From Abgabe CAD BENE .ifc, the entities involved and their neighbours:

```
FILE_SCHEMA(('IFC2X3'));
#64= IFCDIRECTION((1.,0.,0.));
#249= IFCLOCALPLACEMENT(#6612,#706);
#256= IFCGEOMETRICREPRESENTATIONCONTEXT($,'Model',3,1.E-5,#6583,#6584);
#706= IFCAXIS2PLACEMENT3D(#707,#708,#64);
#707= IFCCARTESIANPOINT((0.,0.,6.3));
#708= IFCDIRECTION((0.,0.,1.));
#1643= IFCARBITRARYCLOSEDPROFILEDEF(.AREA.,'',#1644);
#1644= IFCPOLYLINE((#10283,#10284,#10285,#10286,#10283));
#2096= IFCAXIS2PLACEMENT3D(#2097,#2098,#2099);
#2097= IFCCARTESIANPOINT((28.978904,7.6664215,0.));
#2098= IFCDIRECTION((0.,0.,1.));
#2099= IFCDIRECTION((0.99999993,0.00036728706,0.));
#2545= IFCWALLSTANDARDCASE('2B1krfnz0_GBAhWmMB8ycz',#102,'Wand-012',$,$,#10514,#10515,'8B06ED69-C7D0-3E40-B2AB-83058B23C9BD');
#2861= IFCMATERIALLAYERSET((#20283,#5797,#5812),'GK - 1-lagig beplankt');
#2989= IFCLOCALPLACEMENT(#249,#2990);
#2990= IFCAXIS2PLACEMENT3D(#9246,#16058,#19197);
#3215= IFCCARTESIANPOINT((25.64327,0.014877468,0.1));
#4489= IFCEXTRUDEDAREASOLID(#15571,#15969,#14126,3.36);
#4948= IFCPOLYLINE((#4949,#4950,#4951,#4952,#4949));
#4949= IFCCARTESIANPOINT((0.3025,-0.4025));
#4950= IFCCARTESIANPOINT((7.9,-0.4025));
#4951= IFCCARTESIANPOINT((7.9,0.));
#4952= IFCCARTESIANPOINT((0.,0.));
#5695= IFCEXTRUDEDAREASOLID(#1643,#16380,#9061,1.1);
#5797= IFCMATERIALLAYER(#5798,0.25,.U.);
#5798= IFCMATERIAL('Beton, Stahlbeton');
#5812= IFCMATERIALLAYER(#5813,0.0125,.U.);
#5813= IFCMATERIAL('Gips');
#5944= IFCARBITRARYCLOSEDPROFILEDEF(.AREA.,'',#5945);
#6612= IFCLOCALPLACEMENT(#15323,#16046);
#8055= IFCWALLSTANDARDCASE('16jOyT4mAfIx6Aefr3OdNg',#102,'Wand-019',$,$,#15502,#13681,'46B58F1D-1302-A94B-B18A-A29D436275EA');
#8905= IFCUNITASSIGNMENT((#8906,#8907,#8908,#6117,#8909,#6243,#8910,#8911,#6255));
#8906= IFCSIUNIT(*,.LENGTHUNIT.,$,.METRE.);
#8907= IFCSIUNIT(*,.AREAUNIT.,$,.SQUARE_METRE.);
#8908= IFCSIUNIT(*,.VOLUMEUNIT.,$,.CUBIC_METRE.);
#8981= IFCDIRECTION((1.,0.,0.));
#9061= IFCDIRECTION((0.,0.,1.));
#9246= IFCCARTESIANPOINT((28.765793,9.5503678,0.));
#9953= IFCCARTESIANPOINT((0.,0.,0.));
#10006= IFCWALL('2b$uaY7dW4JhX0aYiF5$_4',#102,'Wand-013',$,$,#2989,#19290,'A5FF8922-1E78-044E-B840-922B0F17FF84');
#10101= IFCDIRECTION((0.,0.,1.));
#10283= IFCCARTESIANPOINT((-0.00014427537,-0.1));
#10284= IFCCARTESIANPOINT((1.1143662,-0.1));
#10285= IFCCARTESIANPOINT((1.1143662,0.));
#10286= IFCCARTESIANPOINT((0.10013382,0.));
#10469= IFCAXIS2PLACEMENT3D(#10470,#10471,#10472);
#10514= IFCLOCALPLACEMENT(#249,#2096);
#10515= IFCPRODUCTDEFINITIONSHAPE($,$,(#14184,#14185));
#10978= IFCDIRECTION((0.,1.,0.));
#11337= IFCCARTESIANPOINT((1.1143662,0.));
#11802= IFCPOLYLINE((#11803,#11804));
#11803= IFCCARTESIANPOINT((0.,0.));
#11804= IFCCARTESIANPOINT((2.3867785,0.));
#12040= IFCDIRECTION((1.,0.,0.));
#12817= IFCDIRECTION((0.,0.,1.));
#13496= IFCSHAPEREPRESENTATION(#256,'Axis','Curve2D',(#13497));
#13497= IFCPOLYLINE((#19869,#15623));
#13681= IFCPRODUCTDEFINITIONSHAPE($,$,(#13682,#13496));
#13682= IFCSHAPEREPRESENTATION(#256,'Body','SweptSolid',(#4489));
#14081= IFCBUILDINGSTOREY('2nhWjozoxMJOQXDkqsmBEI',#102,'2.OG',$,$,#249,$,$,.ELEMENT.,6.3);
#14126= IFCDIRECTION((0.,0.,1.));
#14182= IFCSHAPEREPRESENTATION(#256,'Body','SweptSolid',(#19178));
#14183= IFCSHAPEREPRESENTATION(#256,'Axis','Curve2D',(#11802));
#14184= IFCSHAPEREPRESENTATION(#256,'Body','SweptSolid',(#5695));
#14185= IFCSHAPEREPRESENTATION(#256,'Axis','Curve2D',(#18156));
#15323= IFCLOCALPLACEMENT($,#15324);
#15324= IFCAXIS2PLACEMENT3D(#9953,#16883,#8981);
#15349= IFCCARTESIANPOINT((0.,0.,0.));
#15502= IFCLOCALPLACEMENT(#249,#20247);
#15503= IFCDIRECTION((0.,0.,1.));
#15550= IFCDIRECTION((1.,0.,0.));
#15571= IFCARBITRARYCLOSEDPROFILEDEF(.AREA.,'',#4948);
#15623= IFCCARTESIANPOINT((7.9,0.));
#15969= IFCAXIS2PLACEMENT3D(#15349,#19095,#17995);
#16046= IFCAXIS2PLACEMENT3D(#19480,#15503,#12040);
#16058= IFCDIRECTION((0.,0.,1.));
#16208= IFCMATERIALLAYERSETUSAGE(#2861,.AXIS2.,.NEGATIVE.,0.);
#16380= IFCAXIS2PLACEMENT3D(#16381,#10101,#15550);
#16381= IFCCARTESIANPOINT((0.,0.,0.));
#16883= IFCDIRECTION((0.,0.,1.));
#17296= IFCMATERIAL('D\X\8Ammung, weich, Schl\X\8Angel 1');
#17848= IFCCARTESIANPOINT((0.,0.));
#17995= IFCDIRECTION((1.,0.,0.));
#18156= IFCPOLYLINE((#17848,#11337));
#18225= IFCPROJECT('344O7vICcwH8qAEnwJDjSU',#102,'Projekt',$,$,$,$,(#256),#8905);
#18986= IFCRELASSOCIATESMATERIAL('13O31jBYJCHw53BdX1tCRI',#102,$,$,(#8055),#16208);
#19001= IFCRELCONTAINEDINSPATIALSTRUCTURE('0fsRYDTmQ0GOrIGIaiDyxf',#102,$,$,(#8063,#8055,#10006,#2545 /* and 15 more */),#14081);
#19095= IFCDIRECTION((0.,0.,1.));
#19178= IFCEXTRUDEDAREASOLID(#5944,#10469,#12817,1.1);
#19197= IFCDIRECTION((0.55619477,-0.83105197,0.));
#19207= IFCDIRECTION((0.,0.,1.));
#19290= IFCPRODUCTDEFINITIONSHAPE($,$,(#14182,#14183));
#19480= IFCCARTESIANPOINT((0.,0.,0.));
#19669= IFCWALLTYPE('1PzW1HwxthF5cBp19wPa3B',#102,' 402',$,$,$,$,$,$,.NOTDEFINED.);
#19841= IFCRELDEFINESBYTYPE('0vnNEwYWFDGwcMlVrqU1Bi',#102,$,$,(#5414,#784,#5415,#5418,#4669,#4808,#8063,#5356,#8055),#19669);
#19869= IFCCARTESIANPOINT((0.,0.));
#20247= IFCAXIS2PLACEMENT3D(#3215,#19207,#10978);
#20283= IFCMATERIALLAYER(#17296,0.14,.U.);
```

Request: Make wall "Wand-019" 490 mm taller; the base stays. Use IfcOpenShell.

```python
import ifcopenshell
import ifcopenshell.geom
import ifcopenshell.util.shape

model = ifcopenshell.open("Abgabe CAD BENE .ifc")
settings = ifcopenshell.geom.settings()


def volume(element):
    """Net volume in cubic metres, openings subtracted."""
    shape = ifcopenshell.geom.create_shape(settings, element)
    return ifcopenshell.util.shape.get_volume(shape.geometry)


wall = model.by_guid("16jOyT4mAfIx6Aefr3OdNg")
before = volume(wall)

body = next(r for r in wall.Representation.Representations if r.RepresentationIdentifier == "Body")
solid = body.Items[0]
old_height = solid.Depth
solid.Depth += 0.49
after = volume(wall)

print(f"height {old_height:g} -> {solid.Depth:g}, volume {before:.3f} -> {after:.3f} m3")

model.write("Abgabe CAD BENE _v2.ifc")
```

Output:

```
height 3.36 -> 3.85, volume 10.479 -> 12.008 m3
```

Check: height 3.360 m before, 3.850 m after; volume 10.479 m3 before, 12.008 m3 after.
